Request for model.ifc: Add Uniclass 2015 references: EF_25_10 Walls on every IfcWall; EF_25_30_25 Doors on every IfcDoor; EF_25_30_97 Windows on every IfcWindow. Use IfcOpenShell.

First a look at what the model holds.

```python
import ifcopenshell

model = ifcopenshell.open("model.ifc")
print(model.schema)
print("classifications:", [c.Name for c in model.by_type("IfcClassification")])
for ifc_class in ("IfcDoor", "IfcRoof", "IfcStair", "IfcWall", "IfcWindow"):
    print(ifc_class, len(model.by_type(ifc_class)))
```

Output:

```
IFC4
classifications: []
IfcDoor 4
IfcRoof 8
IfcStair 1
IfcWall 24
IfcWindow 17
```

```python
import ifcopenshell
import ifcopenshell.api.classification

model = ifcopenshell.open("model.ifc")

system = ifcopenshell.api.classification.add_classification(model, classification="Uniclass 2015")

codes = {
    "IfcWall": ("EF_25_10", "Walls"),
    "IfcDoor": ("EF_25_30_25", "Doors"),
    "IfcWindow": ("EF_25_30_97", "Windows"),
}
for ifc_class, (code, name) in codes.items():
    products = model.by_type(ifc_class)
    ifcopenshell.api.classification.add_reference(
        model, products=products, classification=system, identification=code, name=name
    )
    print(code, len(products))

model.write("model_rev.ifc")
```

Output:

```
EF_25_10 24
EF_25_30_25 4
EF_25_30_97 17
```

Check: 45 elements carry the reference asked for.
